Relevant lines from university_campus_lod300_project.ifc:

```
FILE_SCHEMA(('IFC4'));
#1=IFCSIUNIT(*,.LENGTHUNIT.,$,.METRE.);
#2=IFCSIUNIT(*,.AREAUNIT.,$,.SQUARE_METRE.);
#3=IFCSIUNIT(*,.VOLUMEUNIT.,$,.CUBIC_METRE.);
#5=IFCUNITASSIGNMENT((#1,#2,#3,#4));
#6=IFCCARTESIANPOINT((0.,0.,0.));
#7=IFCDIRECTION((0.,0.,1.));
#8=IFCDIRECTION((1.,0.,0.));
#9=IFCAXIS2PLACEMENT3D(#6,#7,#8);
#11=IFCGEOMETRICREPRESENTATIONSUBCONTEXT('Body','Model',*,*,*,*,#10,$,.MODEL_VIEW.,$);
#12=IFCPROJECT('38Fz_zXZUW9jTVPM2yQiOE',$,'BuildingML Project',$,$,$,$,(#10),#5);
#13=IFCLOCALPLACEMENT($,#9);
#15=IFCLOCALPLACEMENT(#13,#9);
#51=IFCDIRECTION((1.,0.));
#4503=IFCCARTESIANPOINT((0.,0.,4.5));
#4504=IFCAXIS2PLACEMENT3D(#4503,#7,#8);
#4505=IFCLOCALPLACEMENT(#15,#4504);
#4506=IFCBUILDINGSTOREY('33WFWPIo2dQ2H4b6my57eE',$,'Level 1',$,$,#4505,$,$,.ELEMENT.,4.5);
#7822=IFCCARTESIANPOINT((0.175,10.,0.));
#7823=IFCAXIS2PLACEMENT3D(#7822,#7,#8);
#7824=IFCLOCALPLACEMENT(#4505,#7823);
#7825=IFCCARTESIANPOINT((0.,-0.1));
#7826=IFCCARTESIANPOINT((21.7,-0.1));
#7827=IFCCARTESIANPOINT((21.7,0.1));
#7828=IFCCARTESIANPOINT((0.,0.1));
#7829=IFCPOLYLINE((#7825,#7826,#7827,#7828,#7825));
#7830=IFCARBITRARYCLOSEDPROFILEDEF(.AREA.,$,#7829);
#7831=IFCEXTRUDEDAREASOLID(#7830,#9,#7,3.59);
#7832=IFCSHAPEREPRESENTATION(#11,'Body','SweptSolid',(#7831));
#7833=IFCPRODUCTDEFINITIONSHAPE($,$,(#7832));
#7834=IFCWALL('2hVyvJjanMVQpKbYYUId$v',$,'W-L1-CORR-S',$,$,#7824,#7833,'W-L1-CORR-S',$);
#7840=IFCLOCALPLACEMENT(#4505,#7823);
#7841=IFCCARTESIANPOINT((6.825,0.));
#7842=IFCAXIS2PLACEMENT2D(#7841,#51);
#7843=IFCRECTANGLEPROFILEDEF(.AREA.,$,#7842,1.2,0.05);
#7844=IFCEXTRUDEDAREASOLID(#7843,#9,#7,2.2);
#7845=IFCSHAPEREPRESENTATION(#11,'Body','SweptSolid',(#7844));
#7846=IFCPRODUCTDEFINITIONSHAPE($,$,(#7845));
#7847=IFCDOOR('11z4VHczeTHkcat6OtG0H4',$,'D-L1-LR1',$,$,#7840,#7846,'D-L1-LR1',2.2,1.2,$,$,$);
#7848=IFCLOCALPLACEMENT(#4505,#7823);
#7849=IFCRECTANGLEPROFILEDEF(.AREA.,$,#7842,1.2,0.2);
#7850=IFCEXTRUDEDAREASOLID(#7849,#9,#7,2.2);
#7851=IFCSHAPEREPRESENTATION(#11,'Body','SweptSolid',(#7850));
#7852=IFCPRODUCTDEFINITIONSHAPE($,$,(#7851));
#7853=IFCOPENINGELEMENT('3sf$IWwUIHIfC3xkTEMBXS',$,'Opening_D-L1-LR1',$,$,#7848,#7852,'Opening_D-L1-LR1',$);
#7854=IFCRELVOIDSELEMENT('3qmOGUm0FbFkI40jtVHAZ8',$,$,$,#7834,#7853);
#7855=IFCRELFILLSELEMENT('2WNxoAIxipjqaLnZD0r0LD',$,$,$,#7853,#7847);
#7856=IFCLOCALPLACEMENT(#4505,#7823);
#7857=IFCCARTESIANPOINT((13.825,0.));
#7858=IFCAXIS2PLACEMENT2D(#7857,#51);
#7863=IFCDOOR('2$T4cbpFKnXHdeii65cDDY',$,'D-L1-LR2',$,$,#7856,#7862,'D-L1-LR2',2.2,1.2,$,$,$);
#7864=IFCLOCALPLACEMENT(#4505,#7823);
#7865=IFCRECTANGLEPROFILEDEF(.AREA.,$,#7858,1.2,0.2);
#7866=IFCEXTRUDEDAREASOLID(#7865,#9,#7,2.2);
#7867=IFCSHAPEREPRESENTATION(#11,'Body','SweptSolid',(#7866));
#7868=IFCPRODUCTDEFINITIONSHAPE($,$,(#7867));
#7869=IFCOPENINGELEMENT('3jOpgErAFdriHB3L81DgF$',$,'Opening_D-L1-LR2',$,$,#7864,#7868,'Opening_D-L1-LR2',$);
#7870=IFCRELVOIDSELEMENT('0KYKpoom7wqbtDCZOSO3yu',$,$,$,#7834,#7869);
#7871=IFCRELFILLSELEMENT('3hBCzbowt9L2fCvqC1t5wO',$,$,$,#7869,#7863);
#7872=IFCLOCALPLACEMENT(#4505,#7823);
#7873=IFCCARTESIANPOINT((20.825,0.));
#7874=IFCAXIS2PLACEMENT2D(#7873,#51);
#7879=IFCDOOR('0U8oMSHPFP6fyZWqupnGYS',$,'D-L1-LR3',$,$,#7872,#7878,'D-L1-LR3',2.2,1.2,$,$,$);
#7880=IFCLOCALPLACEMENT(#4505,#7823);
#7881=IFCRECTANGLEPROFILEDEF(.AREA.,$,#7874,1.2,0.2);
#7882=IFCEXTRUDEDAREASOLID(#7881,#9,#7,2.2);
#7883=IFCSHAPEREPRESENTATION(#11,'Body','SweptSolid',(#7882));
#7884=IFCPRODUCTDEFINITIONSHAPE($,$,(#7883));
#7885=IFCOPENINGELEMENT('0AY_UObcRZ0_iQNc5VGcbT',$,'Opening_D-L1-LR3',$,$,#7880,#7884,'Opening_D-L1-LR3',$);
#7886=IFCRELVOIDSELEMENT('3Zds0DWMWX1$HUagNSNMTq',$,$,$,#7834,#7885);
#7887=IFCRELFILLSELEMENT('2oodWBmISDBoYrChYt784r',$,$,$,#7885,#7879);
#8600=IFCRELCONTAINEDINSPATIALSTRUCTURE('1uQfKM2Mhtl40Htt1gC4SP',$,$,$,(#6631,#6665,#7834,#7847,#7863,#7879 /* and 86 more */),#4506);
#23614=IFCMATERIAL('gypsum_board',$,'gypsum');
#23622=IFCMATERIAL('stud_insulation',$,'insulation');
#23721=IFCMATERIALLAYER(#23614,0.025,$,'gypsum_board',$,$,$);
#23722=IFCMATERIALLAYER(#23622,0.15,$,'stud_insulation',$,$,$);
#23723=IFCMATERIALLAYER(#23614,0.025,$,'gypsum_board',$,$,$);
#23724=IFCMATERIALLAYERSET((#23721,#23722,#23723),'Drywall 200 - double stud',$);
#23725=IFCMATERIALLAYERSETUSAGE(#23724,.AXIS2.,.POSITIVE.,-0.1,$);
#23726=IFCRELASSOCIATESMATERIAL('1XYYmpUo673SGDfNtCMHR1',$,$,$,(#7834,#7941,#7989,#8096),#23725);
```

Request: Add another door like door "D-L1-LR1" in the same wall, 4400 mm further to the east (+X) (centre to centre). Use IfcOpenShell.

```python
import ifcopenshell
import ifcopenshell.api.feature
import ifcopenshell.api.geometry
import ifcopenshell.api.root
import ifcopenshell.geom
import ifcopenshell.util.element
import ifcopenshell.util.placement
import ifcopenshell.util.shape
import ifcopenshell.util.unit

model = ifcopenshell.open("university_campus_lod300_project.ifc")
unit_scale = ifcopenshell.util.unit.calculate_unit_scale(model)
settings = ifcopenshell.geom.settings()


def volume(element):
    """Net volume in cubic metres, openings subtracted."""
    shape = ifcopenshell.geom.create_shape(settings, element)
    return ifcopenshell.util.shape.get_volume(shape.geometry)


door = model.by_guid("11z4VHczeTHkcat6OtG0H4")
opening = door.FillsVoids[0].RelatingOpeningElement
wall = opening.VoidsElements[0].RelatingBuildingElement
before = volume(wall)
shift = ifcopenshell.util.placement.get_local_placement(wall.ObjectPlacement)[:3, 0] * 4.4 / unit_scale

# copy_class copies the void relationship, type, container and properties, but no geometry.
new_opening = ifcopenshell.api.root.copy_class(model, product=opening)
new_opening.Representation = ifcopenshell.util.element.copy_deep(
    model, opening.Representation, exclude=["IfcGeometricRepresentationContext", "IfcRepresentationMap"]
)
new_opening.Tag = None
new_door = ifcopenshell.api.root.copy_class(model, product=door)
new_door.Representation = ifcopenshell.util.element.copy_deep(
    model, door.Representation, exclude=["IfcGeometricRepresentationContext", "IfcRepresentationMap"]
)
new_door.Tag = None
ifcopenshell.api.feature.add_filling(model, opening=new_opening, element=new_door)

for old, new in ((opening, new_opening), (door, new_door)):
    matrix = ifcopenshell.util.placement.get_local_placement(old.ObjectPlacement)
    matrix[:3, 3] += shift
    ifcopenshell.api.geometry.edit_object_placement(model, product=new, matrix=matrix, is_si=False)

after = volume(wall)

print(f"wall volume {before:.3f} -> {after:.3f} m3")

model.write("university_campus_lod300_project_updated.ifc")
```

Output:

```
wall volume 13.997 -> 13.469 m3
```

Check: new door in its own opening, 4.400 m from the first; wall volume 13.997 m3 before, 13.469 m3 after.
